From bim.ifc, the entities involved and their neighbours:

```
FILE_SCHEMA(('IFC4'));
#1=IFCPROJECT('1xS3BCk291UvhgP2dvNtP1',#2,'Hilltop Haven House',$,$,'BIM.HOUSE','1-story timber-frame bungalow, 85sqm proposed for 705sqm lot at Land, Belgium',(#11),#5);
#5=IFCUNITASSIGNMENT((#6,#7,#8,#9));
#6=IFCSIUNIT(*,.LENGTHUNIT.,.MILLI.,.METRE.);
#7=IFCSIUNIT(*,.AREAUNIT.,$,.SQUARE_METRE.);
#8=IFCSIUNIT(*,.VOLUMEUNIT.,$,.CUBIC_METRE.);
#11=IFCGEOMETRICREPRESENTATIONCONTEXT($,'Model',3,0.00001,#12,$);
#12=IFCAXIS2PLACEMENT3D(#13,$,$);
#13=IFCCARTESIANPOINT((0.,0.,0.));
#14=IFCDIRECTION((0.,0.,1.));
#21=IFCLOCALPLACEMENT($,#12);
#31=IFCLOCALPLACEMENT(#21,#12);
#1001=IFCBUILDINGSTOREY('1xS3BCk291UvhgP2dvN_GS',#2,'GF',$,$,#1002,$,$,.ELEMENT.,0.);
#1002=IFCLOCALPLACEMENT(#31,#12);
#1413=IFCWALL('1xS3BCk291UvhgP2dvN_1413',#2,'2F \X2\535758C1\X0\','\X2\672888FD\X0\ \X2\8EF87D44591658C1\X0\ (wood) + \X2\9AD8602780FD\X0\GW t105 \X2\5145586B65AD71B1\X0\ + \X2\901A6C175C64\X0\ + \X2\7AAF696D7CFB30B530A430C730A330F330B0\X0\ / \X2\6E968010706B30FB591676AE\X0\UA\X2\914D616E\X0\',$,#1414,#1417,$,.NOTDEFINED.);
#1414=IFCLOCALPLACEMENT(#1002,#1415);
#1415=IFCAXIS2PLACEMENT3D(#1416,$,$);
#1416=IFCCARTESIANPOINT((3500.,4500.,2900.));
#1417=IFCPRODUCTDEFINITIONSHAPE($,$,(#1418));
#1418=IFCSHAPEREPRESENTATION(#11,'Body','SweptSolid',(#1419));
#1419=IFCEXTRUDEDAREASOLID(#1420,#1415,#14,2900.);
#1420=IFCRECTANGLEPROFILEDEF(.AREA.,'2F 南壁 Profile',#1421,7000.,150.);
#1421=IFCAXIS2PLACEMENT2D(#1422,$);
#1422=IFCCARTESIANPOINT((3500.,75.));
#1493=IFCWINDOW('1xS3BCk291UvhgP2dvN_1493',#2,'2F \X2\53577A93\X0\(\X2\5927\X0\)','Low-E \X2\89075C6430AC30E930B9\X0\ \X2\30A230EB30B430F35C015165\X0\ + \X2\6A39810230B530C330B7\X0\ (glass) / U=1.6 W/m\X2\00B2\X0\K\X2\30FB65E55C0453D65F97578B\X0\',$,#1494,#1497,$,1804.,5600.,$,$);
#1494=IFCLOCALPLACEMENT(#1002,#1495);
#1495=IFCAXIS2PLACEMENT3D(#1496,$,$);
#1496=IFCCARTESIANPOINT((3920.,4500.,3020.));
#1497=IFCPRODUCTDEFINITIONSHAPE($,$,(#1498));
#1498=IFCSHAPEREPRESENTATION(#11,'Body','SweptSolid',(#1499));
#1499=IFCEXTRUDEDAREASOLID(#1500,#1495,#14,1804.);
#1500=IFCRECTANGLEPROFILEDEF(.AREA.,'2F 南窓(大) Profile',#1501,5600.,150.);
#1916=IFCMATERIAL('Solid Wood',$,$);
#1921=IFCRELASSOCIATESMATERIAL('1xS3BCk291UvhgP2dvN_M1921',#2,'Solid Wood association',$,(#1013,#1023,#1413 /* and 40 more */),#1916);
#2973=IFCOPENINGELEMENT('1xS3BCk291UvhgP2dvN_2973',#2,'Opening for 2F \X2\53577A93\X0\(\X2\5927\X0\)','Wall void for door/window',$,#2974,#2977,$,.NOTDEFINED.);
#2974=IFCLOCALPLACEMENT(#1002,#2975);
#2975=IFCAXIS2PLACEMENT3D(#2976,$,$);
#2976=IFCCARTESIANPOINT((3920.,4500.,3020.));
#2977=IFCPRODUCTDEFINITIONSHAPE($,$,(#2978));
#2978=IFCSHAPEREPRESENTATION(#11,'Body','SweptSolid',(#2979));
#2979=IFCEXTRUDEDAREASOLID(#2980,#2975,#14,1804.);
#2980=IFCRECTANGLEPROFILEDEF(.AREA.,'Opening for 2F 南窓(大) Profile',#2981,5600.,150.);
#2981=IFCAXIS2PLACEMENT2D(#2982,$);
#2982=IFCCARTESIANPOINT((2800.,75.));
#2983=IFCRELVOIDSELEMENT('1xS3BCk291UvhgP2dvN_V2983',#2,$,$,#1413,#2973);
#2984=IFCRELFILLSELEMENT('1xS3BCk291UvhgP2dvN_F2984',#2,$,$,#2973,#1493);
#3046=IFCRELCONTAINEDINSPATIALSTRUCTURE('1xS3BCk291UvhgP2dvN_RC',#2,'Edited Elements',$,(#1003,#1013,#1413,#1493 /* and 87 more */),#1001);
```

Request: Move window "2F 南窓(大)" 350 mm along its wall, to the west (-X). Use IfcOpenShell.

```python
import ifcopenshell
import ifcopenshell.api.geometry
import ifcopenshell.util.placement
import ifcopenshell.util.unit

model = ifcopenshell.open("bim.ifc")
unit_scale = ifcopenshell.util.unit.calculate_unit_scale(model)

window = model.by_guid("1xS3BCk291UvhgP2dvN_1493")
opening = window.FillsVoids[0].RelatingOpeningElement
wall = opening.VoidsElements[0].RelatingBuildingElement

wall_matrix = ifcopenshell.util.placement.get_local_placement(wall.ObjectPlacement)
shift = wall_matrix[:3, 0] * -0.35 / unit_scale
before = ifcopenshell.util.placement.get_local_placement(window.ObjectPlacement)[:3, 3].copy()

# The window is not placed relative to its opening, so move both.
for product in (opening, window):
    matrix = ifcopenshell.util.placement.get_local_placement(product.ObjectPlacement)
    matrix[:3, 3] += shift
    ifcopenshell.api.geometry.edit_object_placement(model, product=product, matrix=matrix, is_si=False)

after = ifcopenshell.util.placement.get_local_placement(window.ObjectPlacement)[:3, 3]
print("window moved by", (after - before).round(3) + 0.0)

model.write("bim_edited.ifc")
```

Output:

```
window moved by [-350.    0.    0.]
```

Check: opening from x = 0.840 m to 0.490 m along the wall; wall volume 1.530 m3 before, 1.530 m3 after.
